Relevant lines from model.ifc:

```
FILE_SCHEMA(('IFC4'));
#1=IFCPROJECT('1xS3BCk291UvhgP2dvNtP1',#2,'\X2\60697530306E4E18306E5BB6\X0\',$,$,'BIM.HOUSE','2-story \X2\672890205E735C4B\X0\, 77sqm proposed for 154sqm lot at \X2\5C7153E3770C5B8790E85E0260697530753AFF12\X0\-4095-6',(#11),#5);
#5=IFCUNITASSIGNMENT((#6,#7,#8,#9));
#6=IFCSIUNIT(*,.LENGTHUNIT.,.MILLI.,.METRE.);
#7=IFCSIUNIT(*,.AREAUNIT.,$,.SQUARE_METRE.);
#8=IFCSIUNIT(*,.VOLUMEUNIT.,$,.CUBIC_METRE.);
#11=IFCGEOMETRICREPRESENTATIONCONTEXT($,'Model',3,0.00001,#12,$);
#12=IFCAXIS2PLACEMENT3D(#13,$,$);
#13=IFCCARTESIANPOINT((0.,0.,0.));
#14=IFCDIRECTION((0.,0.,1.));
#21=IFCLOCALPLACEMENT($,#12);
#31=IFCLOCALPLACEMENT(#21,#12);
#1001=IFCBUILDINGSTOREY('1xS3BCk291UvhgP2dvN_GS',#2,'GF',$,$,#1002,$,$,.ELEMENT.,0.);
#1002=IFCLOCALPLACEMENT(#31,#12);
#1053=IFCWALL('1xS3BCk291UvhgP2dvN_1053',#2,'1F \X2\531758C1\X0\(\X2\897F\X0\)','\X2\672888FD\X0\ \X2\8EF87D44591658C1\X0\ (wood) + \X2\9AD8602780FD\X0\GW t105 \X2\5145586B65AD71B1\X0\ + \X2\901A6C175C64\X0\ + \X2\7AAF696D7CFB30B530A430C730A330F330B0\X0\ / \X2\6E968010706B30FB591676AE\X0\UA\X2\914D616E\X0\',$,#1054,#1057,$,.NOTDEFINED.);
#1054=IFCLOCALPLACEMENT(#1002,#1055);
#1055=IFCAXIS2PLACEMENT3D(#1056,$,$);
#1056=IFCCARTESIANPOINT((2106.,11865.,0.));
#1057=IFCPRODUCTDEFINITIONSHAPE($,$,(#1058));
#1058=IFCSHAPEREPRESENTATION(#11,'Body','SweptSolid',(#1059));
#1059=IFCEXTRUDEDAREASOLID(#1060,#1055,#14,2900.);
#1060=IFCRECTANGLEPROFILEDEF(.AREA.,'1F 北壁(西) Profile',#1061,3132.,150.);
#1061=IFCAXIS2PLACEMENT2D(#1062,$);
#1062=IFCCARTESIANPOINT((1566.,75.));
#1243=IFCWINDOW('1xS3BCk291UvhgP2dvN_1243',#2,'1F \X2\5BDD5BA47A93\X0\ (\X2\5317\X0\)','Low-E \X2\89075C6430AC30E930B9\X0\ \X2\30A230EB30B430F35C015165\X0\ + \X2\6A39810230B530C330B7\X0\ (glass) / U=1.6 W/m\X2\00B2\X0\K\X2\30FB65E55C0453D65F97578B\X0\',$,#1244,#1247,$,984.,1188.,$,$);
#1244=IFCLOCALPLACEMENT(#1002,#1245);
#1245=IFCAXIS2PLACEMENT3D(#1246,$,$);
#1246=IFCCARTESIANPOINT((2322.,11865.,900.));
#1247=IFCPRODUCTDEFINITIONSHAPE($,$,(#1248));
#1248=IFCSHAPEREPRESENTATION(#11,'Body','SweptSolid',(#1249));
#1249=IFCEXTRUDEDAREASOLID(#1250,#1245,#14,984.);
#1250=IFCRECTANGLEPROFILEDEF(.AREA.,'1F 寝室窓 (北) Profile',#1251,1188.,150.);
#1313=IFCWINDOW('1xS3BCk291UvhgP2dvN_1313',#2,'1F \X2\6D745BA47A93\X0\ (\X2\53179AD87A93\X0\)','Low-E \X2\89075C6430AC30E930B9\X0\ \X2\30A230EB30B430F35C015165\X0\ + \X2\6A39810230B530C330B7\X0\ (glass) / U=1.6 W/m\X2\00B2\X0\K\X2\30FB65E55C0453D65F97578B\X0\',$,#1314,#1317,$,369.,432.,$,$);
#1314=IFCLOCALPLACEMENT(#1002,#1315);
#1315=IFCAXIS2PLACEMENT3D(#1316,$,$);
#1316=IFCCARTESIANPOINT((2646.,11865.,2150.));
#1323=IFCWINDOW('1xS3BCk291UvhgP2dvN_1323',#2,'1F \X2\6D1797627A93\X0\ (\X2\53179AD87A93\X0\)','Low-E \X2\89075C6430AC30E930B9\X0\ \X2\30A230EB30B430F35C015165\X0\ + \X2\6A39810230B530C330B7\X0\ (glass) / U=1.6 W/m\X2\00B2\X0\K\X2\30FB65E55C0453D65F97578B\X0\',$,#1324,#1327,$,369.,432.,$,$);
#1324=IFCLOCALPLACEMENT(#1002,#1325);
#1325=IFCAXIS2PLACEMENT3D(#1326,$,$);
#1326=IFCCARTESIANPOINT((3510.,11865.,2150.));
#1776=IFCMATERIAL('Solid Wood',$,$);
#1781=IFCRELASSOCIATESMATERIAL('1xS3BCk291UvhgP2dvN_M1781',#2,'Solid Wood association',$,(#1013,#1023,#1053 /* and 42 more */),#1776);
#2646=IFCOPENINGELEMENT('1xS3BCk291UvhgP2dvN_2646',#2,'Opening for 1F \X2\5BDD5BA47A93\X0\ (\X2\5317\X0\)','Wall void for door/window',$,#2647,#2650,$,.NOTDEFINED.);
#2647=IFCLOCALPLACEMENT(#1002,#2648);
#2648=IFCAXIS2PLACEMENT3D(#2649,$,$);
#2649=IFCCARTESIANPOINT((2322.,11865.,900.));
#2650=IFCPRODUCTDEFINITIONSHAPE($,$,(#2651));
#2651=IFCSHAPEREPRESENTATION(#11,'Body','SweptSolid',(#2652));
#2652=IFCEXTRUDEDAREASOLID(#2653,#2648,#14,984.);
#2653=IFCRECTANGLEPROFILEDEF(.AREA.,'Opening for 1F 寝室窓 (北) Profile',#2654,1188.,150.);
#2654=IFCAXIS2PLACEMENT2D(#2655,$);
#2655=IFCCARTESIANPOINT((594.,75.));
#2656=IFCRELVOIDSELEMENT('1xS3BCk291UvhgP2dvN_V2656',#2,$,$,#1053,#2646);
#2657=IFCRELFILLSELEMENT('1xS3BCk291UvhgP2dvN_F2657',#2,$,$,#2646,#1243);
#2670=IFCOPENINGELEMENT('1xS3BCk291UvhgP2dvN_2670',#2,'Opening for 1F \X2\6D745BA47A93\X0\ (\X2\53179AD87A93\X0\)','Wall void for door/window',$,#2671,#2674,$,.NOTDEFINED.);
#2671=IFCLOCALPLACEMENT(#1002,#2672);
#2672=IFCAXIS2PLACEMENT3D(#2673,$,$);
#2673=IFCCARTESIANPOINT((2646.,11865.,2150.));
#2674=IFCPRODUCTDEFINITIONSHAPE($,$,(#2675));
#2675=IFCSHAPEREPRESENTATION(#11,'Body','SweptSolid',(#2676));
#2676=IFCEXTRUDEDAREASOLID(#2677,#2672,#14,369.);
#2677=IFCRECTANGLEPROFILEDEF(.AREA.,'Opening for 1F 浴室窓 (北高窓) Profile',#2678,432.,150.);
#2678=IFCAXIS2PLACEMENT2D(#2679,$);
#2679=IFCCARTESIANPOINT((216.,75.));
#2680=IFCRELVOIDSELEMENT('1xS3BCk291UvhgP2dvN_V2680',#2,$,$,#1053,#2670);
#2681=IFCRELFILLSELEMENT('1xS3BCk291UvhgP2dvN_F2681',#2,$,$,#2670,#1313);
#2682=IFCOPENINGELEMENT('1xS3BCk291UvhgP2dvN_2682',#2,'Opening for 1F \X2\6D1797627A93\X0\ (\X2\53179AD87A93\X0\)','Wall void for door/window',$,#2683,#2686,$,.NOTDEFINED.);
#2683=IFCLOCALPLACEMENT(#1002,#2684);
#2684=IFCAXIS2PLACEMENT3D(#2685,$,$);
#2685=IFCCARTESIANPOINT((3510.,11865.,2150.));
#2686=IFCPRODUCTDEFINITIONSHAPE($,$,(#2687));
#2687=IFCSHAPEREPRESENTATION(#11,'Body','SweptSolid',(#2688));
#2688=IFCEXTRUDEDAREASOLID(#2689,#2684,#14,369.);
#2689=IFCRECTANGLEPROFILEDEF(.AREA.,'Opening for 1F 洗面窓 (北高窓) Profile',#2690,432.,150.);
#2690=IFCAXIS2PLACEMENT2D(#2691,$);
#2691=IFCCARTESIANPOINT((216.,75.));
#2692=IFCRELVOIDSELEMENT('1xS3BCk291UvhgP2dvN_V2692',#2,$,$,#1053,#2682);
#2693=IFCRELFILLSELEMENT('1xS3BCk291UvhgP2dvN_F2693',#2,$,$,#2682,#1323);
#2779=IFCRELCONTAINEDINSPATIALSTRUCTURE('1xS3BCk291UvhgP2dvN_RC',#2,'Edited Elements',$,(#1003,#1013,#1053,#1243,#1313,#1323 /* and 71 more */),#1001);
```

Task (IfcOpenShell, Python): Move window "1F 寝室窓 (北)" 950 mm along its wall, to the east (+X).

```python
import ifcopenshell
import ifcopenshell.api.geometry
import ifcopenshell.util.placement
import ifcopenshell.util.unit

model = ifcopenshell.open("model.ifc")
unit_scale = ifcopenshell.util.unit.calculate_unit_scale(model)

window = model.by_id(1243)
opening = window.FillsVoids[0].RelatingOpeningElement
wall = opening.VoidsElements[0].RelatingBuildingElement

wall_matrix = ifcopenshell.util.placement.get_local_placement(wall.ObjectPlacement)
shift = wall_matrix[:3, 0] * 0.95 / unit_scale
before = ifcopenshell.util.placement.get_local_placement(window.ObjectPlacement)[:3, 3].copy()

# The window is not placed relative to its opening, so move both.
for product in (opening, window):
    matrix = ifcopenshell.util.placement.get_local_placement(product.ObjectPlacement)
    matrix[:3, 3] += shift
    ifcopenshell.api.geometry.edit_object_placement(model, product=product, matrix=matrix, is_si=False)

after = ifcopenshell.util.placement.get_local_placement(window.ObjectPlacement)[:3, 3]
print("window moved by", (after - before).round(3) + 0.0)

model.write("model_updated.ifc")
```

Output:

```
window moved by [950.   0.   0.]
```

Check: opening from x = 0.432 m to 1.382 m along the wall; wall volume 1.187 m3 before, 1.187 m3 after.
